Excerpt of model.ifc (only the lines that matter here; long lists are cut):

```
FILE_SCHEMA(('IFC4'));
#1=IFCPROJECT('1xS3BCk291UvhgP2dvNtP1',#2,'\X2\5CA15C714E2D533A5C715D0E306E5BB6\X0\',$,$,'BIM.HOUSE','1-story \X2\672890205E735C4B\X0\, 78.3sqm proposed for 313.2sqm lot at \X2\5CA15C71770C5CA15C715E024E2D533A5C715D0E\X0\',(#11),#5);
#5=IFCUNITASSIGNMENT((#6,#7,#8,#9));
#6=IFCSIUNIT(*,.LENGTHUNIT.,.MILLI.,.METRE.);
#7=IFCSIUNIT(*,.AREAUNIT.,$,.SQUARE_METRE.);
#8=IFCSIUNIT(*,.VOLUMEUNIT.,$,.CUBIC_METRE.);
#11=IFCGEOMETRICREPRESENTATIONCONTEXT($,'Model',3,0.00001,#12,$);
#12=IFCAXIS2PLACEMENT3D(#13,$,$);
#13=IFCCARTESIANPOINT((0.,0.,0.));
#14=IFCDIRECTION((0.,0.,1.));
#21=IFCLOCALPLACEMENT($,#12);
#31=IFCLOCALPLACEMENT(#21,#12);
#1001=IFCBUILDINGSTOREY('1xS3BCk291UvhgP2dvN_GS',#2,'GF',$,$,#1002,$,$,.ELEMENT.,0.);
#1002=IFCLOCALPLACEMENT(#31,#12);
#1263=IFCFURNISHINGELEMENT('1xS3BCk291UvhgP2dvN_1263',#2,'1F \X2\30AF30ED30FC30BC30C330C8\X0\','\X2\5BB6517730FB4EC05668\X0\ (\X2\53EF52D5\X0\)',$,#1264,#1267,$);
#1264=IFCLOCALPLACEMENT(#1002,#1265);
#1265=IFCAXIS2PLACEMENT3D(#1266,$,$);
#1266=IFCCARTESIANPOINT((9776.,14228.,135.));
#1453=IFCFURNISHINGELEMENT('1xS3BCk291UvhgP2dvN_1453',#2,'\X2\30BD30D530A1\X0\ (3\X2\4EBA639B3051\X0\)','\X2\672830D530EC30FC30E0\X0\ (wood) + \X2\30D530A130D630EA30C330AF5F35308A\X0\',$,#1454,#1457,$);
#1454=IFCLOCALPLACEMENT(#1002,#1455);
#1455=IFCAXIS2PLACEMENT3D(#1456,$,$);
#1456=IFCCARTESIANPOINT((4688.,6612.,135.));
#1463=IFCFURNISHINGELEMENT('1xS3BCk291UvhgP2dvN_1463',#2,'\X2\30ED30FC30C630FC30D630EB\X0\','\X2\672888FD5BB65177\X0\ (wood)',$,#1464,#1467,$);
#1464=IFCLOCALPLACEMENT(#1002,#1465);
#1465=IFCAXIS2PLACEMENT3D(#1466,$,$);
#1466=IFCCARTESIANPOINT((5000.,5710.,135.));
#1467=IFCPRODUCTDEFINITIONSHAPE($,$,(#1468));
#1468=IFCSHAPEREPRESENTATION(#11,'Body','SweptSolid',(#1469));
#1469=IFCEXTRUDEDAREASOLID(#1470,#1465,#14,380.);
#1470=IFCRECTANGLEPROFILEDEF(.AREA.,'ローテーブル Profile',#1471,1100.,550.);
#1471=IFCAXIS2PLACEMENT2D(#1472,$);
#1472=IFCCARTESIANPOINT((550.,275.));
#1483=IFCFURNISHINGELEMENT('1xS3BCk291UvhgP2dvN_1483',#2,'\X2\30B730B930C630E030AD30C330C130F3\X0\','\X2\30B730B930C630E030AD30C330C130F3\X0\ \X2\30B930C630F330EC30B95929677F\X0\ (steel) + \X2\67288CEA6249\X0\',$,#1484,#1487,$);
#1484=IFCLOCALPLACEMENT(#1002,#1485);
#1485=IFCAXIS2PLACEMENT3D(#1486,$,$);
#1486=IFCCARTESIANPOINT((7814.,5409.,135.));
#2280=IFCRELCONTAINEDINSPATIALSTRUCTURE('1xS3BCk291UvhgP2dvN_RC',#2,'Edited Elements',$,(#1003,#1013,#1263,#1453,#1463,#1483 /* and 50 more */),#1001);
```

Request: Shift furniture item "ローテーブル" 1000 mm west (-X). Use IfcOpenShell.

```python
import ifcopenshell
import ifcopenshell.api.geometry
import ifcopenshell.util.placement

model = ifcopenshell.open("model.ifc")

item = model.by_guid("1xS3BCk291UvhgP2dvN_1463")
matrix = ifcopenshell.util.placement.get_local_placement(item.ObjectPlacement)
matrix[0, 3] -= 1000.0
ifcopenshell.api.geometry.edit_object_placement(model, product=item, matrix=matrix, is_si=False)

print(ifcopenshell.util.placement.get_local_placement(item.ObjectPlacement).round(3) + 0.0)

model.write("model_rev.ifc")
```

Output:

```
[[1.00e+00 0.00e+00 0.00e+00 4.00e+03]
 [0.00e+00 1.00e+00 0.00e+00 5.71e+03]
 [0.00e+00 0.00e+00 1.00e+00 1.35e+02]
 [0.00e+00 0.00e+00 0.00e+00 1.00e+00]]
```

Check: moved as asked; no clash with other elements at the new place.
